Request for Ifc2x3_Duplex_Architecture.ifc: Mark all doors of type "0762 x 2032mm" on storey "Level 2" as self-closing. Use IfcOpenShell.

First a look at what the model holds.

```python
import ifcopenshell
import ifcopenshell.util.element

model = ifcopenshell.open("Ifc2x3_Duplex_Architecture.ifc")
print(model.schema)
storey = next(s for s in model.by_type("IfcBuildingStorey") if s.Name == "Level 2")
doors = [e for e in ifcopenshell.util.element.get_decomposition(storey) if e.is_a("IfcDoor")]
seen = {}
for e in doors:
    element_type = ifcopenshell.util.element.get_type(e)
    key = (element_type.Name if element_type != e and element_type else None, ifcopenshell.util.element.get_pset(e, "Pset_DoorCommon", "SelfClosing"))
    seen[key] = seen.get(key, 0) + 1
for (name, value), count in sorted(seen.items(), key=str):
    print(count, "x", name, "|", value)
```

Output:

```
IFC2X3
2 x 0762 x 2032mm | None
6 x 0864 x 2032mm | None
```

```python
import ifcopenshell
import ifcopenshell.api.pset
import ifcopenshell.util.element

model = ifcopenshell.open("Ifc2x3_Duplex_Architecture.ifc")

storey = next(s for s in model.by_type("IfcBuildingStorey") if s.Name == "Level 2")
doors = [e for e in ifcopenshell.util.element.get_decomposition(storey) if e.is_a("IfcDoor")]

count = 0
for e in doors:
    element_type = ifcopenshell.util.element.get_type(e)
    if element_type in (None, e) or element_type.Name != "0762 x 2032mm":
        continue
    # add_pset returns the element's existing set when there is one.
    pset = ifcopenshell.api.pset.add_pset(model, product=e, name="Pset_DoorCommon")
    ifcopenshell.api.pset.edit_pset(model, pset=pset, properties={"SelfClosing": True})
    count += 1

print(count, "doors updated")

model.write("Ifc2x3_Duplex_Architecture_v2.ifc")
```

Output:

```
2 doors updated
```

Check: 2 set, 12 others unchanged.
